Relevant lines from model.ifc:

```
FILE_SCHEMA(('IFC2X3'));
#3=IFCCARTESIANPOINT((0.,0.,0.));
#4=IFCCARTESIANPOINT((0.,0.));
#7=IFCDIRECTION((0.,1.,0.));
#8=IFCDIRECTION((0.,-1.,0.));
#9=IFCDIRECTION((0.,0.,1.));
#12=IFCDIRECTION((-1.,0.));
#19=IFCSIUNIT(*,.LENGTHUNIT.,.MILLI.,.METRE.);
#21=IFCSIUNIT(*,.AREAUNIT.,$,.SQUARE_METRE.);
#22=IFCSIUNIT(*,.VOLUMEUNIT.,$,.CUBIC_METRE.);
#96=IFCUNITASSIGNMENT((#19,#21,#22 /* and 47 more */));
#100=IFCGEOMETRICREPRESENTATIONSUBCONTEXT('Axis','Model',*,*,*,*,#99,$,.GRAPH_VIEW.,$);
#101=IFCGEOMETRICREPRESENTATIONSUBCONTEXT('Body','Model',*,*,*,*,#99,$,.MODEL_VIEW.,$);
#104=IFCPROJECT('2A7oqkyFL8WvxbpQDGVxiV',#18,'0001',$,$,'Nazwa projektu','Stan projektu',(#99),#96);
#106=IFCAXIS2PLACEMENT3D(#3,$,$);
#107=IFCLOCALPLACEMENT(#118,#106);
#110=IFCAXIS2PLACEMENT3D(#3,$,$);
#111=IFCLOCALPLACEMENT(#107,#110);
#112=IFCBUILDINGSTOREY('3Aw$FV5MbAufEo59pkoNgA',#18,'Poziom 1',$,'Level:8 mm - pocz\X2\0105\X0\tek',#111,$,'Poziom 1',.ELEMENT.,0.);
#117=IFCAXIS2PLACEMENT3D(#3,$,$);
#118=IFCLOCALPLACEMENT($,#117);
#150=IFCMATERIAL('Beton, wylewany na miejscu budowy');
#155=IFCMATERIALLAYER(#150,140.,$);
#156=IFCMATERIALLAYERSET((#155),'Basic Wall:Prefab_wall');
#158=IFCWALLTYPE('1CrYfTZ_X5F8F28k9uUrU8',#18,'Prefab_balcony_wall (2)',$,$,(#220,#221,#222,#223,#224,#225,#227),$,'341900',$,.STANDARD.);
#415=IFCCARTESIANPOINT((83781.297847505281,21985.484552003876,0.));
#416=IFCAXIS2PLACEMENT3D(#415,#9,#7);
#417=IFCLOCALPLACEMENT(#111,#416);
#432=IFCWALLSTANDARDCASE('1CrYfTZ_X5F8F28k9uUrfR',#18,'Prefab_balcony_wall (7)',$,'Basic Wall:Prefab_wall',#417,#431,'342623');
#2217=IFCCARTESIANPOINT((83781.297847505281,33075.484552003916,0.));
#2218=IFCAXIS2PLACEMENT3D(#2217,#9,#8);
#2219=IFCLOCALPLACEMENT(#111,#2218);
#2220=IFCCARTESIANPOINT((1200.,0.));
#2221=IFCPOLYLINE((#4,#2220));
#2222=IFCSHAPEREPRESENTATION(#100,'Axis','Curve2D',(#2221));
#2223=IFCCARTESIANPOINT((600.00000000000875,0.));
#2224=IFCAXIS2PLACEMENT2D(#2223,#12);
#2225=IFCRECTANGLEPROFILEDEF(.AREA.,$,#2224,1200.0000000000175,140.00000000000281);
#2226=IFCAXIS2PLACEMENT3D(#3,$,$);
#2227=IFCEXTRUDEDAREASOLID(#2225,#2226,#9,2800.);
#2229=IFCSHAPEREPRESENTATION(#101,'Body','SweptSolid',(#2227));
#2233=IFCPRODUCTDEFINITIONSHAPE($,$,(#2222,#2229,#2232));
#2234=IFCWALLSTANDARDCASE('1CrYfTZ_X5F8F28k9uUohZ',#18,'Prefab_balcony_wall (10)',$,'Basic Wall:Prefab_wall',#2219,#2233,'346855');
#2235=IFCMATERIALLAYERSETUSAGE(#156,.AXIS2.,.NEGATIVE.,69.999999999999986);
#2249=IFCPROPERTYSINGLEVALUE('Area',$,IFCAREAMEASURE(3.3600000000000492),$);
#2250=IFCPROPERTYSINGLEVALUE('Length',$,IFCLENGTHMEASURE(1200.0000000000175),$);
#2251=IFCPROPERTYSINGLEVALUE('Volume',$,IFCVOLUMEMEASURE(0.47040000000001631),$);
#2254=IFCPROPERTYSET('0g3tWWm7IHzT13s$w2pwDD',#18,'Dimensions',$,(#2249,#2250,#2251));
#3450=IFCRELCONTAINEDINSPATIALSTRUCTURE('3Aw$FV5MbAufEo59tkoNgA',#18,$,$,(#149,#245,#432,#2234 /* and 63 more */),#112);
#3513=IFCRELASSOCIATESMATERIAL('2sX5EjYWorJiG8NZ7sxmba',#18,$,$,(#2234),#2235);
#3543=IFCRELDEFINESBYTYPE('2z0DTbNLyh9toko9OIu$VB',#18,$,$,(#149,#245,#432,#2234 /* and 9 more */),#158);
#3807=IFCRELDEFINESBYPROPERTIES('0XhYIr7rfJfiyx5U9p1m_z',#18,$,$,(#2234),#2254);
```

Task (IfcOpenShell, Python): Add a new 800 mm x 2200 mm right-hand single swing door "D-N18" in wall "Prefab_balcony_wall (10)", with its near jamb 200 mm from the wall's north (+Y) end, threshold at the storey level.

```python
import numpy as np
import ifcopenshell
import ifcopenshell.api.feature
import ifcopenshell.api.geometry
import ifcopenshell.api.pset
import ifcopenshell.api.root
import ifcopenshell.api.spatial
import ifcopenshell.api.type
import ifcopenshell.geom
import ifcopenshell.util.element
import ifcopenshell.util.placement
import ifcopenshell.util.representation
import ifcopenshell.util.shape
import ifcopenshell.util.unit

model = ifcopenshell.open("model.ifc")
unit_scale = ifcopenshell.util.unit.calculate_unit_scale(model)
area_scale = ifcopenshell.util.unit.calculate_unit_scale(model, "AREAUNIT")
volume_scale = ifcopenshell.util.unit.calculate_unit_scale(model, "VOLUMEUNIT")
settings = ifcopenshell.geom.settings()


def volume(element):
    """Net volume in cubic metres, openings subtracted."""
    shape = ifcopenshell.geom.create_shape(settings, element)
    return ifcopenshell.util.shape.get_volume(shape.geometry)


wall = model.by_id(2234)
storey = ifcopenshell.util.element.get_container(wall, ifc_class="IfcBuildingStorey")
context = ifcopenshell.util.representation.get_context(model, "Model", "Body", "MODEL_VIEW")
before = volume(wall)

width, height, from_end, sill = 0.8, 2.2, 0.2, 0.0  # metres

# The wall runs along its own X axis, and the end named is its -X end.
wall_shape = ifcopenshell.geom.create_shape(settings, wall)
x, y, z = ifcopenshell.util.shape.get_vertices(wall_shape.geometry).T
start = x.min() + from_end
face, thickness = float(y.min()), float(y.max() - y.min())
wall_matrix = ifcopenshell.util.placement.get_local_placement(wall.ObjectPlacement)
level = ifcopenshell.util.placement.get_local_placement(storey.ObjectPlacement)[2, 3]


def in_wall(x, y):
    """Placement at x, y metres in the wall's axes, at sill height."""
    matrix = wall_matrix.copy()
    matrix[:, 3] = wall_matrix @ np.array([x / unit_scale, y / unit_scale, 0.0, 1.0])
    matrix[2, 3] = level + sill / unit_scale
    return matrix


# Opening: a box that overshoots both wall faces by 50 mm.
opening = ifcopenshell.api.root.create_entity(model, ifc_class="IfcOpeningElement")
box = ifcopenshell.api.geometry.add_wall_representation(
    model, context=context, length=width, height=height, thickness=thickness + 0.1
)
ifcopenshell.api.geometry.assign_representation(model, product=opening, representation=box)
ifcopenshell.api.geometry.edit_object_placement(model, product=opening, matrix=in_wall(start, face - 0.05), is_si=False)
ifcopenshell.api.feature.add_feature(model, feature=opening, element=wall)

door = ifcopenshell.api.root.create_entity(model, ifc_class="IfcDoor", name="D-N18")
door.OverallWidth, door.OverallHeight = width / unit_scale, height / unit_scale
body = ifcopenshell.api.geometry.add_door_representation(
    model,
    context=context,
    overall_width=door.OverallWidth,
    overall_height=door.OverallHeight,
    operation_type="SINGLE_SWING_RIGHT",
    lining_properties={"LiningDepth": thickness / unit_scale, "ThresholdDepth": thickness / unit_scale},
)
ifcopenshell.api.geometry.assign_representation(model, product=door, representation=body)
ifcopenshell.api.spatial.assign_container(model, products=[door], relating_structure=storey)
fills = ifcopenshell.api.feature.add_filling(model, opening=opening, element=door)
fills.OwnerHistory = door.OwnerHistory  # required in IFC2X3

# IFC2X3 keeps the operation on the door style.
style = ifcopenshell.api.root.create_entity(model, ifc_class="IfcDoorStyle", name="D-N18")
style.OperationType, style.ConstructionType = "SINGLE_SWING_RIGHT", "NOTDEFINED"
style.ParameterTakesPrecedence = style.Sizeable = False
ifcopenshell.api.type.assign_type(model, related_objects=[door], relating_type=style)

# The lining spans the wall, so the door starts at the wall face.
ifcopenshell.api.geometry.edit_object_placement(model, product=door, matrix=in_wall(start, face), is_si=False)

after = volume(wall)

# Update the wall's stored quantities.
pset = model.by_id(ifcopenshell.util.element.get_pset(wall, "Dimensions", should_inherit=False)["id"])
ifcopenshell.api.pset.edit_pset(model, pset=pset, properties={
    "Area": model.create_entity("IfcAreaMeasure", after / thickness / area_scale),
    "Volume": model.create_entity("IfcVolumeMeasure", after / volume_scale),
})

print(f"wall volume {before:.3f} -> {after:.3f} m3")

model.write("model_v2.ifc")
```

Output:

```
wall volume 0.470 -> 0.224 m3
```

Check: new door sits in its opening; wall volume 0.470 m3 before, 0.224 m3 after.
